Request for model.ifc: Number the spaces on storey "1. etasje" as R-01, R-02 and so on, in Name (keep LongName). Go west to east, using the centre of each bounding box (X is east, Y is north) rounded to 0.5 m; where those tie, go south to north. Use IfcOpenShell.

First a look at what the model holds.

```python
import ifcopenshell
import ifcopenshell.util.element
import ifcopenshell.util.placement

model = ifcopenshell.open("model.ifc")
print(model.schema)
storey = next(s for s in model.by_type("IfcBuildingStorey") if s.Name == "1. etasje")
spaces = [e for e in ifcopenshell.util.element.get_decomposition(storey) if e.is_a("IfcSpace")]
for e in sorted(spaces, key=lambda e: e.id()):
    origin = ifcopenshell.util.placement.get_local_placement(e.ObjectPlacement)[:3, 3]
    print(e.id(), e.Name, e.LongName, origin.round(2) + 0.0, sep=" | ")
```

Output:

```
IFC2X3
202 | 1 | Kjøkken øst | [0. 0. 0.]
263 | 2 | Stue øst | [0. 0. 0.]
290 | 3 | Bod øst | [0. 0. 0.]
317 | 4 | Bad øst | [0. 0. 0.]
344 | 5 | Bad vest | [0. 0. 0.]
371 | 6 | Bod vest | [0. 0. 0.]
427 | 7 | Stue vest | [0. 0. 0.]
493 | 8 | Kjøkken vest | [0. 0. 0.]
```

```python
import ifcopenshell
import ifcopenshell.geom
import ifcopenshell.util.element
import ifcopenshell.util.shape

model = ifcopenshell.open("model.ifc")
settings = ifcopenshell.geom.settings()
settings.set("use-world-coords", True)


def centre(element):
    shape = ifcopenshell.geom.create_shape(settings, element)
    return ifcopenshell.util.shape.get_bbox_centroid(shape.geometry)


storey = next(s for s in model.by_type("IfcBuildingStorey") if s.Name == "1. etasje")
spaces = [e for e in ifcopenshell.util.element.get_decomposition(storey) if e.is_a("IfcSpace")]

# Insertion points can sit at a corner or the storey origin, so sort by the geometry (in metres).
centres = {e: centre(e) for e in spaces}
spaces.sort(key=lambda e: (round(centres[e][0] / 0.5), centres[e][1]))

for i, e in enumerate(spaces, start=1):
    number = f"R-{i:02d}"
    e.Name = number
    print(e.id(), number)

model.write("model_rev.ifc")
```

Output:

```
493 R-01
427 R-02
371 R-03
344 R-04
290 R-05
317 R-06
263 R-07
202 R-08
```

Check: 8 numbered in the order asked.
